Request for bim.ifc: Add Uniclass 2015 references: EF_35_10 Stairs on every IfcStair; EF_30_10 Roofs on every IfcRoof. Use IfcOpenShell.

First a look at what the model holds.

```python
import ifcopenshell

model = ifcopenshell.open("bim.ifc")
print(model.schema)
print("classifications:", [c.Name for c in model.by_type("IfcClassification")])
for ifc_class in ("IfcDoor", "IfcRoof", "IfcStair", "IfcWall", "IfcWindow"):
    print(ifc_class, len(model.by_type(ifc_class)))
```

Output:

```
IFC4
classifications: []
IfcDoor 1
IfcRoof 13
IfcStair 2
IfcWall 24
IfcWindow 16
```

```python
import ifcopenshell
import ifcopenshell.api.classification

model = ifcopenshell.open("bim.ifc")

system = ifcopenshell.api.classification.add_classification(model, classification="Uniclass 2015")

codes = {
    "IfcStair": ("EF_35_10", "Stairs"),
    "IfcRoof": ("EF_30_10", "Roofs"),
}
for ifc_class, (code, name) in codes.items():
    products = model.by_type(ifc_class)
    ifcopenshell.api.classification.add_reference(
        model, products=products, classification=system, identification=code, name=name
    )
    print(code, len(products))

model.write("bim_updated.ifc")
```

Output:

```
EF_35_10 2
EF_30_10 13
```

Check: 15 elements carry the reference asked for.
